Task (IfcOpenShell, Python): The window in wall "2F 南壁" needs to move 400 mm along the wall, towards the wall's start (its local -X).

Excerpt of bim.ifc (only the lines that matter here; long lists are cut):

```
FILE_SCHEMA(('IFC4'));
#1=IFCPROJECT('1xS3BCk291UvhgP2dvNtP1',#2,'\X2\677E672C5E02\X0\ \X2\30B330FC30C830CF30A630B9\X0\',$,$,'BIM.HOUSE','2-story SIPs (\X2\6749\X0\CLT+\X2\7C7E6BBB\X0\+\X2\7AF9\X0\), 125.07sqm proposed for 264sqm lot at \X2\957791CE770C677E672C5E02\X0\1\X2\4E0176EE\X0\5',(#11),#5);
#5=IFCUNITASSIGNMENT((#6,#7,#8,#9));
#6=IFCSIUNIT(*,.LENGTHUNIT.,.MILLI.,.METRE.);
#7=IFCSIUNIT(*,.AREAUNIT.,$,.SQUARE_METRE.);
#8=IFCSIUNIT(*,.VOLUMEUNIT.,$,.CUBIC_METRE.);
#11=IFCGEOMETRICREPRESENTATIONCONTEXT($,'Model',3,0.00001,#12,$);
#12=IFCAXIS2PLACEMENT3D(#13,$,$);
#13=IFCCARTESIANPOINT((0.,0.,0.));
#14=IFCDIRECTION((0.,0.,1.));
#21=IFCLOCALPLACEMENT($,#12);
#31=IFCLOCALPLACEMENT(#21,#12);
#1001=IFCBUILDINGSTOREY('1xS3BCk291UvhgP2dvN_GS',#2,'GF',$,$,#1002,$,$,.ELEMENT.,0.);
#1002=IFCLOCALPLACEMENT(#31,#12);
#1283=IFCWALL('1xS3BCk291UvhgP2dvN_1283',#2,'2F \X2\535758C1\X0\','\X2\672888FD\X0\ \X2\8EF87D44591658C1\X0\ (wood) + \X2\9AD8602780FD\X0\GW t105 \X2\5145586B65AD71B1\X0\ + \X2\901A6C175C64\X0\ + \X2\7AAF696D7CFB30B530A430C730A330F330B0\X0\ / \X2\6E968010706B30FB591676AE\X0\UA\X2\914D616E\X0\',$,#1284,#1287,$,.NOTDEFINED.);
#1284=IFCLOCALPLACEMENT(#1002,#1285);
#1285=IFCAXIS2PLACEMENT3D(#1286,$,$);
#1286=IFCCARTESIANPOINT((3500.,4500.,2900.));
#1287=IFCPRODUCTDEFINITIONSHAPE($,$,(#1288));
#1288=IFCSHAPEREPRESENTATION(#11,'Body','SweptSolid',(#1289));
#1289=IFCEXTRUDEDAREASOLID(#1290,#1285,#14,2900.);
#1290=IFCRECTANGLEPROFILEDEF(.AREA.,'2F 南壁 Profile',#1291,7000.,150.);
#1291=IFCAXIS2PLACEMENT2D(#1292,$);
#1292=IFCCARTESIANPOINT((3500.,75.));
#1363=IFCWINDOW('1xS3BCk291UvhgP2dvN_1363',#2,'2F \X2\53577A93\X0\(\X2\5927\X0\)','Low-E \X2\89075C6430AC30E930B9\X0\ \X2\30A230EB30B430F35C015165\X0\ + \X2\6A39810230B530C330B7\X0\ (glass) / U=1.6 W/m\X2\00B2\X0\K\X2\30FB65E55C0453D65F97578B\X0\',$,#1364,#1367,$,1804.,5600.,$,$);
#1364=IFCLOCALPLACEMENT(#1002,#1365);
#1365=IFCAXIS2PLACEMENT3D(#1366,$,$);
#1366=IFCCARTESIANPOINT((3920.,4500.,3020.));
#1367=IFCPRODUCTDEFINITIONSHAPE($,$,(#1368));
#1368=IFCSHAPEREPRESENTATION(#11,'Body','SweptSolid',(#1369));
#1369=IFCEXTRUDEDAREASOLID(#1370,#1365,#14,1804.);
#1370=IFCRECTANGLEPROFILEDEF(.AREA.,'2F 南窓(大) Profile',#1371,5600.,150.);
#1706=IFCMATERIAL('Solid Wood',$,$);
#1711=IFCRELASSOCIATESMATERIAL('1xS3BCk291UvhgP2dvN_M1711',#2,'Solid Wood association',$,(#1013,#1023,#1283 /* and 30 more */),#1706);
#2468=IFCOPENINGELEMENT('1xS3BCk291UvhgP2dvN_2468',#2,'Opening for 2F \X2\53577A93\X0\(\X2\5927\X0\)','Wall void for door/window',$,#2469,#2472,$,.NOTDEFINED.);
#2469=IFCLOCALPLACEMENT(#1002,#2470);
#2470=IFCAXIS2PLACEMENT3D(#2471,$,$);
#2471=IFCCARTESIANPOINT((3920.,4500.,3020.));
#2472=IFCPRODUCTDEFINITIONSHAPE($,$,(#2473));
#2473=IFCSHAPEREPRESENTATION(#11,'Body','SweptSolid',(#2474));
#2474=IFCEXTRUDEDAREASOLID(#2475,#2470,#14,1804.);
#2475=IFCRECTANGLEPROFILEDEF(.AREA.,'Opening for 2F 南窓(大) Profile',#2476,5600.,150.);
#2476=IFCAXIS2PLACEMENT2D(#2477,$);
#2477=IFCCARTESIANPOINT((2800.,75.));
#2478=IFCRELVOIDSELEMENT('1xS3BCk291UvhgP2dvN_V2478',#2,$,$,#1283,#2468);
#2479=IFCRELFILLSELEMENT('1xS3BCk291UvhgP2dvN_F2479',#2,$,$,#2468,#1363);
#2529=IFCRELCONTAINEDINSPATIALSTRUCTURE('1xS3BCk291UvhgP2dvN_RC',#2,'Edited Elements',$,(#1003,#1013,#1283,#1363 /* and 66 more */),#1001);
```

```python
import ifcopenshell
import ifcopenshell.api.geometry
import ifcopenshell.util.placement

model = ifcopenshell.open("bim.ifc")

window = model.by_guid("1xS3BCk291UvhgP2dvN_1363")
opening = window.FillsVoids[0].RelatingOpeningElement
wall = opening.VoidsElements[0].RelatingBuildingElement

wall_matrix = ifcopenshell.util.placement.get_local_placement(wall.ObjectPlacement)
shift = wall_matrix[:3, 0] * -400.0
before = ifcopenshell.util.placement.get_local_placement(window.ObjectPlacement)[:3, 3].copy()

# The window is not placed relative to its opening, so move both.
for product in (opening, window):
    matrix = ifcopenshell.util.placement.get_local_placement(product.ObjectPlacement)
    matrix[:3, 3] += shift
    ifcopenshell.api.geometry.edit_object_placement(model, product=product, matrix=matrix, is_si=False)

after = ifcopenshell.util.placement.get_local_placement(window.ObjectPlacement)[:3, 3]
print("window moved by", (after - before).round(3) + 0.0)

model.write("bim_rev.ifc")
```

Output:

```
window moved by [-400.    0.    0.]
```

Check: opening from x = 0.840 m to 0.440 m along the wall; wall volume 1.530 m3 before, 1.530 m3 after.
